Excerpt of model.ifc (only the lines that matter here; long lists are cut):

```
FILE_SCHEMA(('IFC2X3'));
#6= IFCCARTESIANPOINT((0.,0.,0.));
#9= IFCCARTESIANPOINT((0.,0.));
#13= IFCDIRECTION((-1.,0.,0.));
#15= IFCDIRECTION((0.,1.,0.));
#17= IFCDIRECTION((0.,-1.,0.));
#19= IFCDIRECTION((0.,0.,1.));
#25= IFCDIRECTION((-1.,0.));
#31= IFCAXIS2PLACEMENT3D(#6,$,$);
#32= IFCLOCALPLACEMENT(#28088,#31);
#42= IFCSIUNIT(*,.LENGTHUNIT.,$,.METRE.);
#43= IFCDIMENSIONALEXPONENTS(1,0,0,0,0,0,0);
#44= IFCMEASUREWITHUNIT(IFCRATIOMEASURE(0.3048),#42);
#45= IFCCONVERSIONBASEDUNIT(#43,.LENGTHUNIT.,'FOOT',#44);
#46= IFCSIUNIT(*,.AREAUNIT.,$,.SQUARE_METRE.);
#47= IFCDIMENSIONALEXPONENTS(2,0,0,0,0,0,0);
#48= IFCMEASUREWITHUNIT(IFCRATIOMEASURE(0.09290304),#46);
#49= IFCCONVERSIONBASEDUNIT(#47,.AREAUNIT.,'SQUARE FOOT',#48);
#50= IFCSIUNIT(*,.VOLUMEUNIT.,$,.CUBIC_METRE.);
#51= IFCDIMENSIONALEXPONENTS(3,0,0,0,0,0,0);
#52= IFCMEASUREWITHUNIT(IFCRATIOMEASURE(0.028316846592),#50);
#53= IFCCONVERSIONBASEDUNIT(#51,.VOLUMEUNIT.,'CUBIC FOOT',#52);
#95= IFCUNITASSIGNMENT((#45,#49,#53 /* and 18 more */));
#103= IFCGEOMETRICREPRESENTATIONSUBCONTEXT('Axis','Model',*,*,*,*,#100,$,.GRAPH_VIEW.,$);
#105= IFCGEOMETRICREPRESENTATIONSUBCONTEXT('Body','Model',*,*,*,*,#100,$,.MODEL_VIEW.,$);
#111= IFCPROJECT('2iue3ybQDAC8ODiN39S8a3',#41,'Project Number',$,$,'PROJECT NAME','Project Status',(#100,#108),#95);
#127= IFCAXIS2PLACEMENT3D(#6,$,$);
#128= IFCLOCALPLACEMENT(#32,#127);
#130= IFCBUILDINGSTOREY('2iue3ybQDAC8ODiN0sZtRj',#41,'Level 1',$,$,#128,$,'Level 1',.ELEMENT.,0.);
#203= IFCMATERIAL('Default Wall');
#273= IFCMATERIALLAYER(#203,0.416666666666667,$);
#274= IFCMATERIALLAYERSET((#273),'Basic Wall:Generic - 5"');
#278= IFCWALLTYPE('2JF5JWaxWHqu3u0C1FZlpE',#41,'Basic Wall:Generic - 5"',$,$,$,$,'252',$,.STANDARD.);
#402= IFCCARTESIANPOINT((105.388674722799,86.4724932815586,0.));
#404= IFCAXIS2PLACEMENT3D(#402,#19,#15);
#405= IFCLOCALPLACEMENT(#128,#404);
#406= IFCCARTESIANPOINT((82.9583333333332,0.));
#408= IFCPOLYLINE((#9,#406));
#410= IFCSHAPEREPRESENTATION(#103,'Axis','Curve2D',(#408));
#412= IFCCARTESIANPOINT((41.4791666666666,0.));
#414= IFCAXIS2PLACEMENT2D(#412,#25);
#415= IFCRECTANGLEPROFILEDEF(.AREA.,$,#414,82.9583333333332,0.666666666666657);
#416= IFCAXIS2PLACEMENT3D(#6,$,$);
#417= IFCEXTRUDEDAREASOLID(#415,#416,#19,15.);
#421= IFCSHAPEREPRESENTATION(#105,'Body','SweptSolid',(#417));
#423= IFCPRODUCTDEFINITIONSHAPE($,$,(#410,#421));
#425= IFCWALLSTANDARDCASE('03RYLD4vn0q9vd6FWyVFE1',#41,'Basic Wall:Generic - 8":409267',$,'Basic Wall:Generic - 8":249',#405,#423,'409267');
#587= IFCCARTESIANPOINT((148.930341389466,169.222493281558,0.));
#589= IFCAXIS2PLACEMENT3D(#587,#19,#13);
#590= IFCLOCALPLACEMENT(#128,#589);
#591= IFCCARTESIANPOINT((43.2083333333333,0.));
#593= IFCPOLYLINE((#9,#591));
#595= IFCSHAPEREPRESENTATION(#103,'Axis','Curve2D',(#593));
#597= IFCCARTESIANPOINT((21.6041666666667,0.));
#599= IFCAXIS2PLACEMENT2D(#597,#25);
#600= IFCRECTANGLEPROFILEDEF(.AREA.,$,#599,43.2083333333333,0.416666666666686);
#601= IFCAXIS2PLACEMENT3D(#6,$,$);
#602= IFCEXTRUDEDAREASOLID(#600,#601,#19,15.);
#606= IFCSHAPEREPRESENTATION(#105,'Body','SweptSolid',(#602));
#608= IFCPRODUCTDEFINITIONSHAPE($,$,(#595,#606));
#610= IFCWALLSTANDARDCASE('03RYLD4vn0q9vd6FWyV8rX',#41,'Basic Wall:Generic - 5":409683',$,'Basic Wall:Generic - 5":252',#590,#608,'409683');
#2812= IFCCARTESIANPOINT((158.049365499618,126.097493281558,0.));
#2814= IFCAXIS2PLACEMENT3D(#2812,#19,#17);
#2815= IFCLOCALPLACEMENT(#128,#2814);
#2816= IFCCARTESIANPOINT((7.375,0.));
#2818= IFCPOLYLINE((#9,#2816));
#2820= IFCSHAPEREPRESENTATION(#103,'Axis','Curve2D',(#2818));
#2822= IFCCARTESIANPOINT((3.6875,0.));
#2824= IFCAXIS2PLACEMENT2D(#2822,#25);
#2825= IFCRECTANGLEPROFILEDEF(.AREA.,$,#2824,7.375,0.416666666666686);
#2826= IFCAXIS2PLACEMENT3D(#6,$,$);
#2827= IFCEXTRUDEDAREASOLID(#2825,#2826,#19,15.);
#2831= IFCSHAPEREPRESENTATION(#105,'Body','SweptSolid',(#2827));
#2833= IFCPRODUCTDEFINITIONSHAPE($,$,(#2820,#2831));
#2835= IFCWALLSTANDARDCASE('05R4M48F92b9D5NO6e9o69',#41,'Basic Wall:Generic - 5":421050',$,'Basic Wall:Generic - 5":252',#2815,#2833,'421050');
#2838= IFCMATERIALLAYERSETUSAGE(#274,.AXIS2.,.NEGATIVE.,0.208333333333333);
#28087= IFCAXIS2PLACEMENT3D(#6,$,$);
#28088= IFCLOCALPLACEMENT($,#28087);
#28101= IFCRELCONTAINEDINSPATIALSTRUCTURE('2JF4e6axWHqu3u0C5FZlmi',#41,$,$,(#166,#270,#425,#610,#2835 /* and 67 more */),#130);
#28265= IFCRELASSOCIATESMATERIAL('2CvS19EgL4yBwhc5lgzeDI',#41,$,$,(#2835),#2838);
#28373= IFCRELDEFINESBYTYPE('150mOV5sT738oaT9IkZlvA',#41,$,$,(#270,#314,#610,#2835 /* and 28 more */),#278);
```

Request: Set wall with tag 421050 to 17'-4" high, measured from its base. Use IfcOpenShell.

```python
import ifcopenshell
import ifcopenshell.geom
import ifcopenshell.util.representation
import ifcopenshell.util.shape
import ifcopenshell.util.unit

model = ifcopenshell.open("model.ifc")
unit_scale = ifcopenshell.util.unit.calculate_unit_scale(model)
settings = ifcopenshell.geom.settings()


def volume(element):
    """Net volume in cubic metres, openings subtracted."""
    shape = ifcopenshell.geom.create_shape(settings, element)
    return ifcopenshell.util.shape.get_volume(shape.geometry)


wall = model.by_guid("05R4M48F92b9D5NO6e9o69")
before = volume(wall)

body = ifcopenshell.util.representation.get_representation(wall, "Model", "Body")
solid = body.Items[0]
old_height = solid.Depth
solid.Depth = 208 * 0.0254 / unit_scale
after = volume(wall)

print(f"height {old_height:g} -> {solid.Depth:g}, volume {before:.3f} -> {after:.3f} m3")

model.write("model_updated.ifc")
```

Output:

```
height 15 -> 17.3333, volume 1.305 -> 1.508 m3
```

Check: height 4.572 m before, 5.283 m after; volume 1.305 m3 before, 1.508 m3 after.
